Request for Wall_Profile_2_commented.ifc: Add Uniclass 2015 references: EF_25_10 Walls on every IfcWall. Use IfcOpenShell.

First a look at what the model holds.

```python
import ifcopenshell

model = ifcopenshell.open("Wall_Profile_2_commented.ifc")
print(model.schema)
print("classifications:", [c.Name for c in model.by_type("IfcClassification")])
for ifc_class in ("IfcDoor", "IfcRoof", "IfcStair", "IfcWall", "IfcWindow"):
    print(ifc_class, len(model.by_type(ifc_class)))
```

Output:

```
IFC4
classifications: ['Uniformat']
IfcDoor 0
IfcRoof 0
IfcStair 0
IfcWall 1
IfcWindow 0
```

```python
import ifcopenshell
import ifcopenshell.api.classification

model = ifcopenshell.open("Wall_Profile_2_commented.ifc")

system = ifcopenshell.api.classification.add_classification(model, classification="Uniclass 2015")

codes = {
    "IfcWall": ("EF_25_10", "Walls"),
}
for ifc_class, (code, name) in codes.items():
    products = model.by_type(ifc_class)
    ifcopenshell.api.classification.add_reference(
        model, products=products, classification=system, identification=code, name=name
    )
    print(code, len(products))

model.write("Wall_Profile_2_commented_v2.ifc")
```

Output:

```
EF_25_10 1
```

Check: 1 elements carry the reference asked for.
